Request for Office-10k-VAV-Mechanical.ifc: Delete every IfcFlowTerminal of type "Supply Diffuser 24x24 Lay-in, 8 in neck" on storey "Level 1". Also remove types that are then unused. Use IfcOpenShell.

First a look at what the model holds.

```python
import ifcopenshell
import ifcopenshell.util.element

model = ifcopenshell.open("Office-10k-VAV-Mechanical.ifc")
print(model.schema)
storey = next(s for s in model.by_type("IfcBuildingStorey") if s.Name == "Level 1")
terminals = [e for e in ifcopenshell.util.element.get_decomposition(storey) if e.is_a("IfcFlowTerminal")]
seen = {}
for e in terminals:
    element_type = ifcopenshell.util.element.get_type(e)
    name = element_type.Name if element_type not in (None, e) else None
    seen[name] = seen.get(name, 0) + 1
for name, count in sorted(seen.items(), key=str):
    print(count, "x", name)
```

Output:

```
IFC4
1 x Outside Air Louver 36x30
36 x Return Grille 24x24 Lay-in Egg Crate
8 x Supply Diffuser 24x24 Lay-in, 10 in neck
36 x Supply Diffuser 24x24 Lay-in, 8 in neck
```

```python
import ifcopenshell
import ifcopenshell.api.root
import ifcopenshell.util.element

model = ifcopenshell.open("Office-10k-VAV-Mechanical.ifc")

storey = next(s for s in model.by_type("IfcBuildingStorey") if s.Name == "Level 1")
terminals = [e for e in ifcopenshell.util.element.get_decomposition(storey) if e.is_a("IfcFlowTerminal")]
targets = [e for e in terminals if (t := ifcopenshell.util.element.get_type(e)) not in (None, e) and t.Name == "Supply Diffuser 24x24 Lay-in, 8 in neck"]
types = {ifcopenshell.util.element.get_type(e) for e in targets} - {None, *targets}

for e in targets:
    ifcopenshell.api.root.remove_product(model, product=e)
print(len(targets), "removed")

unused = [t for t in types if not ifcopenshell.util.element.get_types(t)]
for t in unused:
    ifcopenshell.api.root.remove_product(model, product=t)
print(len(unused), "unused types removed")

model.write("Office-10k-VAV-Mechanical-out.ifc")
```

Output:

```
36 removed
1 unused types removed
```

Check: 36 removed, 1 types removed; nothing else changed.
